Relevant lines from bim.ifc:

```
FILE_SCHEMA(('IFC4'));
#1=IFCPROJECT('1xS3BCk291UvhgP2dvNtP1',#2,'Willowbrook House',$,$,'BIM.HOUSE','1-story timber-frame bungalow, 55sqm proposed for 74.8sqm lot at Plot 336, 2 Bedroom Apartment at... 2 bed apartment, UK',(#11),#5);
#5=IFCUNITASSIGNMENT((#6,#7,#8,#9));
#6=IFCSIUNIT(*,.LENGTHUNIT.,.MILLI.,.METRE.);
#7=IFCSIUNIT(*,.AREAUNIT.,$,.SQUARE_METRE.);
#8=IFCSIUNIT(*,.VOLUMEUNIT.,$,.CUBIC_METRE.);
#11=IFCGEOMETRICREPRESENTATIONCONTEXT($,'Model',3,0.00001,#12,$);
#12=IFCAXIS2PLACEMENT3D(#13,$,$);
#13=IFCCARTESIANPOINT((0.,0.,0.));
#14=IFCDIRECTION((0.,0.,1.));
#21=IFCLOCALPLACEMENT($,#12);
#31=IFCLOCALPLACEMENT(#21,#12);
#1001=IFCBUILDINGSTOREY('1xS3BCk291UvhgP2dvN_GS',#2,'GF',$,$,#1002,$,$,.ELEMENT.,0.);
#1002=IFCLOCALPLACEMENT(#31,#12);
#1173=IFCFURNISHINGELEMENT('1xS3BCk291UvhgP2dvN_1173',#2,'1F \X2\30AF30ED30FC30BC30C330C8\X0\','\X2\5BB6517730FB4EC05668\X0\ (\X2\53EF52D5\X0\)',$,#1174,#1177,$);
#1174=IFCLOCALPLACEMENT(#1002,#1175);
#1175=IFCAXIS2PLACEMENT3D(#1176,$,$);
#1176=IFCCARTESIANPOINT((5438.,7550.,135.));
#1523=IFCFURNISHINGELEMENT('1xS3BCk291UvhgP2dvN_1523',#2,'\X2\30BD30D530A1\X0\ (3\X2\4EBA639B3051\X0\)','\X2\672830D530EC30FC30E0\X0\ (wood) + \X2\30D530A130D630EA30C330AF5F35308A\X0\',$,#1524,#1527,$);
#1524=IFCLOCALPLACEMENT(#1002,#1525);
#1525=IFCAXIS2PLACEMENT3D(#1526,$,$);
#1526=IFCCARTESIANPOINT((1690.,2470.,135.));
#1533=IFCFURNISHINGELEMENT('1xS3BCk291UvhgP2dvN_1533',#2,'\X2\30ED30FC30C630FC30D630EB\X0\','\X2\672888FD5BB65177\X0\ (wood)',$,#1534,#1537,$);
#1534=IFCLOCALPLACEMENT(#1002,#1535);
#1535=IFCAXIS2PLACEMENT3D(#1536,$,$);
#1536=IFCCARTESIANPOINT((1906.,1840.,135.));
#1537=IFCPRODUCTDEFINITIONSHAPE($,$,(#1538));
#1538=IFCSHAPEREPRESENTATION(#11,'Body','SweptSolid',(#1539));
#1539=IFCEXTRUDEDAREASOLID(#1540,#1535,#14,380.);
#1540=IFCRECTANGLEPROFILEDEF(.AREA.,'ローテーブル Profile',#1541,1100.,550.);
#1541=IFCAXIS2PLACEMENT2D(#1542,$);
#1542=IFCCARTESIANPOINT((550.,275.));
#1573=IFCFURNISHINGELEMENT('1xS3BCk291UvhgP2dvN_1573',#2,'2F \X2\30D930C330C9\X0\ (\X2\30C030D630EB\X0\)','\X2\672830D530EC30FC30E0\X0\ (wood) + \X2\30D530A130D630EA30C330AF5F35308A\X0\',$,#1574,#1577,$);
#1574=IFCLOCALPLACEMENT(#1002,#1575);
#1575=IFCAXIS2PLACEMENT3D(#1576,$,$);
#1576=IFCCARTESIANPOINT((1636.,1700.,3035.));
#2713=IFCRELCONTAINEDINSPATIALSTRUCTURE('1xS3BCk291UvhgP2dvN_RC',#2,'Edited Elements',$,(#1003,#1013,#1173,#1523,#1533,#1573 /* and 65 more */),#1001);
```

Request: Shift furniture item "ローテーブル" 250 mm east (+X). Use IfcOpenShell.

```python
import ifcopenshell
import ifcopenshell.api.geometry
import ifcopenshell.util.placement
import ifcopenshell.util.unit

model = ifcopenshell.open("bim.ifc")
unit_scale = ifcopenshell.util.unit.calculate_unit_scale(model)

item = model.by_guid("1xS3BCk291UvhgP2dvN_1533")
matrix = ifcopenshell.util.placement.get_local_placement(item.ObjectPlacement)
matrix[0, 3] += 0.25 / unit_scale
ifcopenshell.api.geometry.edit_object_placement(model, product=item, matrix=matrix, is_si=False)

print(ifcopenshell.util.placement.get_local_placement(item.ObjectPlacement).round(3) + 0.0)

model.write("bim-out.ifc")
```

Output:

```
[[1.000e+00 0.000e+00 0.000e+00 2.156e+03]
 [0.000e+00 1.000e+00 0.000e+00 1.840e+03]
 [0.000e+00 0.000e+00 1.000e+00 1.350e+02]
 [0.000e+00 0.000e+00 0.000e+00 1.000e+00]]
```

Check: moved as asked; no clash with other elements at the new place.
